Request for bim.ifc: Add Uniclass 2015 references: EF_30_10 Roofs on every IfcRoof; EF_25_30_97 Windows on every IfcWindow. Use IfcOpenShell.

First a look at what the model holds.

```python
import ifcopenshell

model = ifcopenshell.open("bim.ifc")
print(model.schema)
print("classifications:", [c.Name for c in model.by_type("IfcClassification")])
for ifc_class in ("IfcDoor", "IfcRoof", "IfcStair", "IfcWall", "IfcWindow"):
    print(ifc_class, len(model.by_type(ifc_class)))
```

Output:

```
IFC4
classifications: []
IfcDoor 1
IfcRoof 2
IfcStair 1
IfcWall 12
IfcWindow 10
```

```python
import ifcopenshell
import ifcopenshell.api.classification

model = ifcopenshell.open("bim.ifc")

system = ifcopenshell.api.classification.add_classification(model, classification="Uniclass 2015")

codes = {
    "IfcRoof": ("EF_30_10", "Roofs"),
    "IfcWindow": ("EF_25_30_97", "Windows"),
}
for ifc_class, (code, name) in codes.items():
    products = model.by_type(ifc_class)
    ifcopenshell.api.classification.add_reference(
        model, products=products, classification=system, identification=code, name=name
    )
    print(code, len(products))

model.write("bim_rev.ifc")
```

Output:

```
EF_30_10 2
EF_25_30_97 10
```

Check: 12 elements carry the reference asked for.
